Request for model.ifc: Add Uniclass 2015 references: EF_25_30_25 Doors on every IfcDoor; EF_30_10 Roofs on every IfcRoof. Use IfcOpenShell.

First a look at what the model holds.

```python
import ifcopenshell

model = ifcopenshell.open("model.ifc")
print(model.schema)
print("classifications:", [c.Name for c in model.by_type("IfcClassification")])
for ifc_class in ("IfcDoor", "IfcRoof", "IfcStair", "IfcWall", "IfcWindow"):
    print(ifc_class, len(model.by_type(ifc_class)))
```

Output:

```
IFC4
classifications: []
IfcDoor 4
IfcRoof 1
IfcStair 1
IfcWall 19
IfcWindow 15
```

```python
import ifcopenshell
import ifcopenshell.api.classification

model = ifcopenshell.open("model.ifc")

system = ifcopenshell.api.classification.add_classification(model, classification="Uniclass 2015")

codes = {
    "IfcDoor": ("EF_25_30_25", "Doors"),
    "IfcRoof": ("EF_30_10", "Roofs"),
}
for ifc_class, (code, name) in codes.items():
    products = model.by_type(ifc_class)
    ifcopenshell.api.classification.add_reference(
        model, products=products, classification=system, identification=code, name=name
    )
    print(code, len(products))

model.write("model_updated.ifc")
```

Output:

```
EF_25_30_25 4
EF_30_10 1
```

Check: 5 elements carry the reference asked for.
